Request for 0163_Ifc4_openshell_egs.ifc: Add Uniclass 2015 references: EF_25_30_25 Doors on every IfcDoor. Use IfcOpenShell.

First a look at what the model holds.

```python
import ifcopenshell

model = ifcopenshell.open("0163_Ifc4_openshell_egs.ifc")
print(model.schema)
print("classifications:", [c.Name for c in model.by_type("IfcClassification")])
for ifc_class in ("IfcDoor", "IfcRoof", "IfcStair", "IfcWall", "IfcWindow"):
    print(ifc_class, len(model.by_type(ifc_class)))
```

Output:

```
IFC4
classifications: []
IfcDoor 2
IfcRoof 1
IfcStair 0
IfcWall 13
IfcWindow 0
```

```python
import ifcopenshell
import ifcopenshell.api.classification

model = ifcopenshell.open("0163_Ifc4_openshell_egs.ifc")

system = ifcopenshell.api.classification.add_classification(model, classification="Uniclass 2015")

codes = {
    "IfcDoor": ("EF_25_30_25", "Doors"),
}
for ifc_class, (code, name) in codes.items():
    products = model.by_type(ifc_class)
    ifcopenshell.api.classification.add_reference(
        model, products=products, classification=system, identification=code, name=name
    )
    print(code, len(products))

model.write("0163_Ifc4_openshell_egs_edited.ifc")
```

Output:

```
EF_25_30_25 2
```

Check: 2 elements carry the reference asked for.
